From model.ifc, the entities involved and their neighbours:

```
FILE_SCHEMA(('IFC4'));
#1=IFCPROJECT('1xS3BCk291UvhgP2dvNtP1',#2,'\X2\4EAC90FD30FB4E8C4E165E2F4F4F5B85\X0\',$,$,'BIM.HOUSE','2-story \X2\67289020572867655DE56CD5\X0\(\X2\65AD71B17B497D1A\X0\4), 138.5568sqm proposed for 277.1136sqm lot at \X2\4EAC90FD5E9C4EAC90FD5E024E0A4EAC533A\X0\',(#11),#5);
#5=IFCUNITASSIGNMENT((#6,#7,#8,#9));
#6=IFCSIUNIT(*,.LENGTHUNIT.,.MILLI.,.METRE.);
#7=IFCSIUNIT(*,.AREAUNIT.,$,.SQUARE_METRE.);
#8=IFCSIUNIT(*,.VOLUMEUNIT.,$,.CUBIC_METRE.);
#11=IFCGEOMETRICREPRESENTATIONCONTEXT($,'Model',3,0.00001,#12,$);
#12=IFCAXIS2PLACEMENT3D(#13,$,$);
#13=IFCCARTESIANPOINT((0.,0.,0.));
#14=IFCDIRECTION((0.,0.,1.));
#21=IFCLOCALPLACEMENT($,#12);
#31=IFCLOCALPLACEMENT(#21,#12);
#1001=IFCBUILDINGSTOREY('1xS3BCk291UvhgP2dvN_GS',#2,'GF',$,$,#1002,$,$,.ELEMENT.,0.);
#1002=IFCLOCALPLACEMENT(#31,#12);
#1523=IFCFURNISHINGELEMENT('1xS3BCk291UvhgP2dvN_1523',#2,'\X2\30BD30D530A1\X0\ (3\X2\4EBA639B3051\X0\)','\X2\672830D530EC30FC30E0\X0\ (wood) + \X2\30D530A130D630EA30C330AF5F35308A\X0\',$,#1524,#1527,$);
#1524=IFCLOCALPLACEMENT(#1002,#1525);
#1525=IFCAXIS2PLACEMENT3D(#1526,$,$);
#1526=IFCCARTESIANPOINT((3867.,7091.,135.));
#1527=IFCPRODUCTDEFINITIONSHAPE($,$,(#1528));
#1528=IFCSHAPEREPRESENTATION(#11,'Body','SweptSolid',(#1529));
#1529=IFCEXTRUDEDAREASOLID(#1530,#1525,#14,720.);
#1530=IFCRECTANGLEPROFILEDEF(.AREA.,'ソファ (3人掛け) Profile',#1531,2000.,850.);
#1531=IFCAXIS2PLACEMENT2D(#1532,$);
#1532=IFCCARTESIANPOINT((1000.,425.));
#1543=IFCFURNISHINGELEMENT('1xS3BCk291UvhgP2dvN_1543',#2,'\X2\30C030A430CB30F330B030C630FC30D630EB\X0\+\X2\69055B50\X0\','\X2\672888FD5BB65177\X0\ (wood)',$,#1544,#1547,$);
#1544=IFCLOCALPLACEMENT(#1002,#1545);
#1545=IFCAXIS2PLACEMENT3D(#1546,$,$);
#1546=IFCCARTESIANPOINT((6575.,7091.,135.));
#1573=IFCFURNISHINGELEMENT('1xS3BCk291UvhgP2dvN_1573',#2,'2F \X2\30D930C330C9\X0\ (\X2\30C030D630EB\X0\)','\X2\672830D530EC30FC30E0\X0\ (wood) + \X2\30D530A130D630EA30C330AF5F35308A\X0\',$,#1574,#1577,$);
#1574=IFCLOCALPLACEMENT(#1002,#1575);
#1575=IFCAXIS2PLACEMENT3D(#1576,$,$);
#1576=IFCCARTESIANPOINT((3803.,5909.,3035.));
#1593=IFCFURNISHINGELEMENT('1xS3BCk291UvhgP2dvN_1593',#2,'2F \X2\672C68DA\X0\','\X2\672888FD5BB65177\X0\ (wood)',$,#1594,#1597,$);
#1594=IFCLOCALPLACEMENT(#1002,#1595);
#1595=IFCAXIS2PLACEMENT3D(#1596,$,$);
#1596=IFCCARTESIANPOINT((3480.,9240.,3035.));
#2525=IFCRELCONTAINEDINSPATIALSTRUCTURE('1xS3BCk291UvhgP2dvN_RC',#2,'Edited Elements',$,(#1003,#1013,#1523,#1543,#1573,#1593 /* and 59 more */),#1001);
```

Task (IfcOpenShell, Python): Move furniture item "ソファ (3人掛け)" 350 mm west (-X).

```python
import ifcopenshell
import ifcopenshell.api.geometry
import ifcopenshell.util.placement
import ifcopenshell.util.unit

model = ifcopenshell.open("model.ifc")
unit_scale = ifcopenshell.util.unit.calculate_unit_scale(model)

item = model.by_guid("1xS3BCk291UvhgP2dvN_1523")
matrix = ifcopenshell.util.placement.get_local_placement(item.ObjectPlacement)
matrix[0, 3] -= 0.35 / unit_scale
ifcopenshell.api.geometry.edit_object_placement(model, product=item, matrix=matrix, is_si=False)

print(ifcopenshell.util.placement.get_local_placement(item.ObjectPlacement).round(3) + 0.0)

model.write("model_updated.ifc")
```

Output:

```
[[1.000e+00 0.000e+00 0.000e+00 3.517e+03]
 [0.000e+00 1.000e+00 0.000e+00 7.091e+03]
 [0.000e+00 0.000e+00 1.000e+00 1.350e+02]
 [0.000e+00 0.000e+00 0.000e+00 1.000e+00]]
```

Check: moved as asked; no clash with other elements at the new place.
